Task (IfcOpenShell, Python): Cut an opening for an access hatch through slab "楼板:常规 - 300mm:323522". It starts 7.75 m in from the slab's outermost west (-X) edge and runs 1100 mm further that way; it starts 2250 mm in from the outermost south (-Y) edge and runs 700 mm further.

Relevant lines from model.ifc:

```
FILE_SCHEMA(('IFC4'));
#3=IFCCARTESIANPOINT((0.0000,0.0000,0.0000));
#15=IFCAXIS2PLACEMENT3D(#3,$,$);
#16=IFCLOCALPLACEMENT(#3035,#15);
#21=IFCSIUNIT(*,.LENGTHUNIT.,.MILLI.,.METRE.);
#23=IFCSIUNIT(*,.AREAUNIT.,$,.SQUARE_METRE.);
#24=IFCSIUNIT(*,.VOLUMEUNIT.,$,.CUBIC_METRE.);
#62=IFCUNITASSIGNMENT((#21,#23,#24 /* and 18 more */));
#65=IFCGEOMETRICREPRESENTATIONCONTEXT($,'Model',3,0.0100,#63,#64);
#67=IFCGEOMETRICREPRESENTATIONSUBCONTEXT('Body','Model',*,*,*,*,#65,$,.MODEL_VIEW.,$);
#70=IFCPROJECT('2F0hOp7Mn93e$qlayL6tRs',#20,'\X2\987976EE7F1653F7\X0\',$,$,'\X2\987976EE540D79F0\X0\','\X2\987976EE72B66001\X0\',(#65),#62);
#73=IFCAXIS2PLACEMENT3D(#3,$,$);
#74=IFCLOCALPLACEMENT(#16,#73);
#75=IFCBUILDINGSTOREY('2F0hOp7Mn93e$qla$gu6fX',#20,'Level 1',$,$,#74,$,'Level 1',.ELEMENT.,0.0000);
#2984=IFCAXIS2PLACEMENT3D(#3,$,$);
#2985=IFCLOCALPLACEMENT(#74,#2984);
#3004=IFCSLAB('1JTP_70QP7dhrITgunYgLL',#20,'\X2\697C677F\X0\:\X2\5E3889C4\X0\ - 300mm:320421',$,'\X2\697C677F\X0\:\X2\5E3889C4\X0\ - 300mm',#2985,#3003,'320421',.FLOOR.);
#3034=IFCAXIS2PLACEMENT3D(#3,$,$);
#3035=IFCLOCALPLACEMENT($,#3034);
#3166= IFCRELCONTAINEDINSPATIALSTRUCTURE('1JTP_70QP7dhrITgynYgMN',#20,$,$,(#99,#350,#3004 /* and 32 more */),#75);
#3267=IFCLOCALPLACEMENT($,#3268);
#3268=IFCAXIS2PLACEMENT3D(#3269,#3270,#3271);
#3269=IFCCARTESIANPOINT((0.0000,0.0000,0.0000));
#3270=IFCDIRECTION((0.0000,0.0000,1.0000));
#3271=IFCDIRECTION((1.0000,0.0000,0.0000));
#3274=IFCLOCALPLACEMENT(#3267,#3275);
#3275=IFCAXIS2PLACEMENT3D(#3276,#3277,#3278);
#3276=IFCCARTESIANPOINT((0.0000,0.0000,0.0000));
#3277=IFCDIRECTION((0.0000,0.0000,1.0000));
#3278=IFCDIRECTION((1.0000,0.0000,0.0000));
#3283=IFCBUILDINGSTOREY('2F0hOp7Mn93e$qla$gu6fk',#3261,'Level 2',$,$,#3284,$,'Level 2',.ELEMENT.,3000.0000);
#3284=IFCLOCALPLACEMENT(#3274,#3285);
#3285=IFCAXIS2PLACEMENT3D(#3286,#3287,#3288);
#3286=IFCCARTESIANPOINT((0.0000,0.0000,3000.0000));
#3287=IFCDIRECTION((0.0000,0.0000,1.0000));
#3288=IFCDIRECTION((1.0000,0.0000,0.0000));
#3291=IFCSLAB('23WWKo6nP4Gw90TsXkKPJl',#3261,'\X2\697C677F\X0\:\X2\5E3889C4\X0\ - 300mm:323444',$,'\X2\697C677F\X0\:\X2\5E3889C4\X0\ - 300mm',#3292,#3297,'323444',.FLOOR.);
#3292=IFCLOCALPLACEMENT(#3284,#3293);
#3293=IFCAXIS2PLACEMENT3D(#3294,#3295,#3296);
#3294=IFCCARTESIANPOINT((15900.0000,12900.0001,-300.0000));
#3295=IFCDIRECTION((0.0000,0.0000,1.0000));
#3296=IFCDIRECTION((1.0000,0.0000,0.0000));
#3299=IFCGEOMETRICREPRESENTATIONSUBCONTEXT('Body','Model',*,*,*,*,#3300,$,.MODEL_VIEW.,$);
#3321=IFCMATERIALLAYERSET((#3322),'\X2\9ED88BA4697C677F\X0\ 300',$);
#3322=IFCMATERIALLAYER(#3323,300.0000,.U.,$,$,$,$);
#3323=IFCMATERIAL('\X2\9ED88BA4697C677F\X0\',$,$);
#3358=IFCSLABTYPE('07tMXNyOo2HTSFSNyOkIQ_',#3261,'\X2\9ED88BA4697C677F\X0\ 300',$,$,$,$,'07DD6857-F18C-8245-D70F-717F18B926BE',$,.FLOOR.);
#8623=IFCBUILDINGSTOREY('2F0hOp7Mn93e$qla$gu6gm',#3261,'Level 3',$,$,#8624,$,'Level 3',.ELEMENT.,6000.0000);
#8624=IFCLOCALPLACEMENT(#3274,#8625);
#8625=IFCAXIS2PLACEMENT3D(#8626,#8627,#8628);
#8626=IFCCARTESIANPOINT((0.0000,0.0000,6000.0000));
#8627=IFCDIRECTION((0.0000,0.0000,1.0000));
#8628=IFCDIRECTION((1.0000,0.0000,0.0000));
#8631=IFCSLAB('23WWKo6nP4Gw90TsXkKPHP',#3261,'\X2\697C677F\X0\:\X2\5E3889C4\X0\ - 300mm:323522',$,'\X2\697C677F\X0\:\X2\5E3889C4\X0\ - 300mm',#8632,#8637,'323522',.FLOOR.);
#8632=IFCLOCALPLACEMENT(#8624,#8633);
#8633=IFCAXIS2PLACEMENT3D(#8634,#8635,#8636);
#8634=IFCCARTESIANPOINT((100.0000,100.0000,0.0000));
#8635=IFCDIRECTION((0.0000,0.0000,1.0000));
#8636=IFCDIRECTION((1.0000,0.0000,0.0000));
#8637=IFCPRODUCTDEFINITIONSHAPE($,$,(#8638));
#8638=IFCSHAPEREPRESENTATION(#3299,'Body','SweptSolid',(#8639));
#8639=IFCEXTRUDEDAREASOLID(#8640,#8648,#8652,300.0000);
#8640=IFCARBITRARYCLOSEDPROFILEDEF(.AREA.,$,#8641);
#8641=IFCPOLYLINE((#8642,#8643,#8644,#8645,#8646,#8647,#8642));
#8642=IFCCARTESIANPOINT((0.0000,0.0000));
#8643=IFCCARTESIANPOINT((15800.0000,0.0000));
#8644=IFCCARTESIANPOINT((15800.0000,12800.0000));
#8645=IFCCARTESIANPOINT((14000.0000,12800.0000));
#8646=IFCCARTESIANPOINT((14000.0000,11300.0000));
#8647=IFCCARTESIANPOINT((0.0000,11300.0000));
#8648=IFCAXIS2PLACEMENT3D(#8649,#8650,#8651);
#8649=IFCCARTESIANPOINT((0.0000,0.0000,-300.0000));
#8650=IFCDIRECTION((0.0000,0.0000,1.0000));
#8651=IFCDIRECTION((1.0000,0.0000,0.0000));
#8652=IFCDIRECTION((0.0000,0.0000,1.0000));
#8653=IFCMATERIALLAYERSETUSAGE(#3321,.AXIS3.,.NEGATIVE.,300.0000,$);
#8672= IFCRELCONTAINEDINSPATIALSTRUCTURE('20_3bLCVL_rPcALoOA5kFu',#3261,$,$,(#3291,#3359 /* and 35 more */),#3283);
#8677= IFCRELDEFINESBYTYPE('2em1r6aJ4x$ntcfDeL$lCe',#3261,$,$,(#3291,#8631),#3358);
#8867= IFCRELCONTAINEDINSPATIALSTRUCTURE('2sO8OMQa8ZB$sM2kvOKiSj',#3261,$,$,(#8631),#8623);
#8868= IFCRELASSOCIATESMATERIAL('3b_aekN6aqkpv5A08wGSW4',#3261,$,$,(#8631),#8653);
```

```python
import numpy as np
import ifcopenshell
import ifcopenshell.api.feature
import ifcopenshell.api.geometry
import ifcopenshell.api.root
import ifcopenshell.geom
import ifcopenshell.util.placement
import ifcopenshell.util.representation
import ifcopenshell.util.shape
import ifcopenshell.util.unit

model = ifcopenshell.open("model.ifc")
unit_scale = ifcopenshell.util.unit.calculate_unit_scale(model)
settings = ifcopenshell.geom.settings()


def volume(element):
    """Net volume in cubic metres, openings subtracted."""
    shape = ifcopenshell.geom.create_shape(settings, element)
    return ifcopenshell.util.shape.get_volume(shape.geometry)


slab = model.by_guid("23WWKo6nP4Gw90TsXkKPHP")
before = volume(slab)

# Extent in the slab's own axes, in metres. The edges named are its -X and -Y sides.
slab_shape = ifcopenshell.geom.create_shape(settings, slab)
vertices = ifcopenshell.util.shape.get_vertices(slab_shape.geometry)
x_min, y_min, bottom = vertices.min(axis=0)
top = vertices[:, 2].max()

opening = ifcopenshell.api.root.create_entity(model, ifc_class="IfcOpeningElement", name="Access hatch opening", predefined_type="OPENING")
context = ifcopenshell.util.representation.get_context(model, "Model", "Body", "MODEL_VIEW")
width, depth = 1.1, 0.7
outline = [(0.0, 0.0), (width, 0.0), (width, depth), (0.0, depth), (0.0, 0.0)]
# Overshoot both faces by 50 mm so the cut is clean.
shape = ifcopenshell.api.geometry.add_slab_representation(
    model, context=context, depth=top - bottom + 0.1, polyline=outline
)
ifcopenshell.api.geometry.assign_representation(model, product=opening, representation=shape)

matrix = ifcopenshell.util.placement.get_local_placement(slab.ObjectPlacement)
matrix[:, 3] = matrix @ np.append(np.array([x_min + 7.75, y_min + 2.25, bottom - 0.05]) / unit_scale, 1.0)
ifcopenshell.api.geometry.edit_object_placement(model, product=opening, matrix=matrix, is_si=False)
ifcopenshell.api.feature.add_feature(model, feature=opening, element=slab)

after = volume(slab)

print(f"slab volume {before:.3f} -> {after:.3f} m3")

model.write("model_updated.ifc")
```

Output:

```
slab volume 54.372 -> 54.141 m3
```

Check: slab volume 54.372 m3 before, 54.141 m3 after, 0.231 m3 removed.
